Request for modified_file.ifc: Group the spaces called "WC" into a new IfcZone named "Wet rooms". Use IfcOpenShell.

First a look at what the model holds.

```python
import ifcopenshell

model = ifcopenshell.open("modified_file.ifc")
print(model.schema)
seen = {}
for space in model.by_type("IfcSpace"):
    seen[space.LongName] = seen.get(space.LongName, 0) + 1
for name, count in sorted(seen.items(), key=str):
    print(count, "x", name)
print("zones:", [z.Name for z in model.by_type("IfcZone")][:20])
```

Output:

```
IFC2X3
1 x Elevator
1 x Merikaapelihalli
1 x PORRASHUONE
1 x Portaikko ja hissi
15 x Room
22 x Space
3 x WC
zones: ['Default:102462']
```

```python
import ifcopenshell
import ifcopenshell.api.group
import ifcopenshell.api.root

model = ifcopenshell.open("modified_file.ifc")

names = {"WC"}
spaces = [s for s in model.by_type("IfcSpace") if s.LongName in names]

zone = ifcopenshell.api.root.create_entity(model, ifc_class="IfcZone", name="Wet rooms")
ifcopenshell.api.group.assign_group(model, products=spaces, group=zone)
print(len(spaces), "spaces in", zone.Name)

model.write("modified_file_updated.ifc")
```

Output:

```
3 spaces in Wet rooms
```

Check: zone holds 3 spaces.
